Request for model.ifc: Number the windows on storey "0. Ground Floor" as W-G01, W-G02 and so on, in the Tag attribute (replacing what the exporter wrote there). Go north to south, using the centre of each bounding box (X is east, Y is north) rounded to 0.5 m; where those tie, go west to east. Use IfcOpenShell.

First a look at what the model holds.

```python
import ifcopenshell
import ifcopenshell.util.element
import ifcopenshell.util.placement

model = ifcopenshell.open("model.ifc")
print(model.schema)
storey = next(s for s in model.by_type("IfcBuildingStorey") if s.Name == "0. Ground Floor")
windows = [e for e in ifcopenshell.util.element.get_decomposition(storey) if e.is_a("IfcWindow")]
for e in sorted(windows, key=lambda e: e.id()):
    origin = ifcopenshell.util.placement.get_local_placement(e.ObjectPlacement)[:3, 3]
    print(e.id(), e.Tag, e.Name, origin.round(2) + 0.0, sep=" | ")
```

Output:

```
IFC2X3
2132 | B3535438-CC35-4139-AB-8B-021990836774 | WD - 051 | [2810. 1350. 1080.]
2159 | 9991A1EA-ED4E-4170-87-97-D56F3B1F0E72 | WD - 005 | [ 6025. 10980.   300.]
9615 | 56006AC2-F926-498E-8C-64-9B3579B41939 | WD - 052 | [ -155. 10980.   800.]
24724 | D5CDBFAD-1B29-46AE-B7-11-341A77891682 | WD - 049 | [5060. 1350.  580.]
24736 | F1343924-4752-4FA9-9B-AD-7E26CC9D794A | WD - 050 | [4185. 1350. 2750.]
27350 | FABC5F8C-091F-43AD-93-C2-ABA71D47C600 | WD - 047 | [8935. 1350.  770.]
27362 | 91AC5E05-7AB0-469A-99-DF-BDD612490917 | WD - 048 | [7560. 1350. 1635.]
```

```python
import ifcopenshell
import ifcopenshell.geom
import ifcopenshell.util.element
import ifcopenshell.util.shape

model = ifcopenshell.open("model.ifc")
settings = ifcopenshell.geom.settings()
settings.set("use-world-coords", True)


def centre(element):
    shape = ifcopenshell.geom.create_shape(settings, element)
    return ifcopenshell.util.shape.get_bbox_centroid(shape.geometry)


storey = next(s for s in model.by_type("IfcBuildingStorey") if s.Name == "0. Ground Floor")
windows = [e for e in ifcopenshell.util.element.get_decomposition(storey) if e.is_a("IfcWindow")]

# Insertion points can sit at a corner or the storey origin, so sort by the geometry (in metres).
centres = {e: centre(e) for e in windows}
windows.sort(key=lambda e: (-round(centres[e][1] / 0.5), centres[e][0]))

for i, e in enumerate(windows, start=1):
    number = f"W-G{i:02d}"
    e.Tag = number
    print(e.id(), number)

model.write("model_updated.ifc")
```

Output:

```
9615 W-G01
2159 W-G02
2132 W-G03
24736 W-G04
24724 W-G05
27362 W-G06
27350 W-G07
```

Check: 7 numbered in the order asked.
